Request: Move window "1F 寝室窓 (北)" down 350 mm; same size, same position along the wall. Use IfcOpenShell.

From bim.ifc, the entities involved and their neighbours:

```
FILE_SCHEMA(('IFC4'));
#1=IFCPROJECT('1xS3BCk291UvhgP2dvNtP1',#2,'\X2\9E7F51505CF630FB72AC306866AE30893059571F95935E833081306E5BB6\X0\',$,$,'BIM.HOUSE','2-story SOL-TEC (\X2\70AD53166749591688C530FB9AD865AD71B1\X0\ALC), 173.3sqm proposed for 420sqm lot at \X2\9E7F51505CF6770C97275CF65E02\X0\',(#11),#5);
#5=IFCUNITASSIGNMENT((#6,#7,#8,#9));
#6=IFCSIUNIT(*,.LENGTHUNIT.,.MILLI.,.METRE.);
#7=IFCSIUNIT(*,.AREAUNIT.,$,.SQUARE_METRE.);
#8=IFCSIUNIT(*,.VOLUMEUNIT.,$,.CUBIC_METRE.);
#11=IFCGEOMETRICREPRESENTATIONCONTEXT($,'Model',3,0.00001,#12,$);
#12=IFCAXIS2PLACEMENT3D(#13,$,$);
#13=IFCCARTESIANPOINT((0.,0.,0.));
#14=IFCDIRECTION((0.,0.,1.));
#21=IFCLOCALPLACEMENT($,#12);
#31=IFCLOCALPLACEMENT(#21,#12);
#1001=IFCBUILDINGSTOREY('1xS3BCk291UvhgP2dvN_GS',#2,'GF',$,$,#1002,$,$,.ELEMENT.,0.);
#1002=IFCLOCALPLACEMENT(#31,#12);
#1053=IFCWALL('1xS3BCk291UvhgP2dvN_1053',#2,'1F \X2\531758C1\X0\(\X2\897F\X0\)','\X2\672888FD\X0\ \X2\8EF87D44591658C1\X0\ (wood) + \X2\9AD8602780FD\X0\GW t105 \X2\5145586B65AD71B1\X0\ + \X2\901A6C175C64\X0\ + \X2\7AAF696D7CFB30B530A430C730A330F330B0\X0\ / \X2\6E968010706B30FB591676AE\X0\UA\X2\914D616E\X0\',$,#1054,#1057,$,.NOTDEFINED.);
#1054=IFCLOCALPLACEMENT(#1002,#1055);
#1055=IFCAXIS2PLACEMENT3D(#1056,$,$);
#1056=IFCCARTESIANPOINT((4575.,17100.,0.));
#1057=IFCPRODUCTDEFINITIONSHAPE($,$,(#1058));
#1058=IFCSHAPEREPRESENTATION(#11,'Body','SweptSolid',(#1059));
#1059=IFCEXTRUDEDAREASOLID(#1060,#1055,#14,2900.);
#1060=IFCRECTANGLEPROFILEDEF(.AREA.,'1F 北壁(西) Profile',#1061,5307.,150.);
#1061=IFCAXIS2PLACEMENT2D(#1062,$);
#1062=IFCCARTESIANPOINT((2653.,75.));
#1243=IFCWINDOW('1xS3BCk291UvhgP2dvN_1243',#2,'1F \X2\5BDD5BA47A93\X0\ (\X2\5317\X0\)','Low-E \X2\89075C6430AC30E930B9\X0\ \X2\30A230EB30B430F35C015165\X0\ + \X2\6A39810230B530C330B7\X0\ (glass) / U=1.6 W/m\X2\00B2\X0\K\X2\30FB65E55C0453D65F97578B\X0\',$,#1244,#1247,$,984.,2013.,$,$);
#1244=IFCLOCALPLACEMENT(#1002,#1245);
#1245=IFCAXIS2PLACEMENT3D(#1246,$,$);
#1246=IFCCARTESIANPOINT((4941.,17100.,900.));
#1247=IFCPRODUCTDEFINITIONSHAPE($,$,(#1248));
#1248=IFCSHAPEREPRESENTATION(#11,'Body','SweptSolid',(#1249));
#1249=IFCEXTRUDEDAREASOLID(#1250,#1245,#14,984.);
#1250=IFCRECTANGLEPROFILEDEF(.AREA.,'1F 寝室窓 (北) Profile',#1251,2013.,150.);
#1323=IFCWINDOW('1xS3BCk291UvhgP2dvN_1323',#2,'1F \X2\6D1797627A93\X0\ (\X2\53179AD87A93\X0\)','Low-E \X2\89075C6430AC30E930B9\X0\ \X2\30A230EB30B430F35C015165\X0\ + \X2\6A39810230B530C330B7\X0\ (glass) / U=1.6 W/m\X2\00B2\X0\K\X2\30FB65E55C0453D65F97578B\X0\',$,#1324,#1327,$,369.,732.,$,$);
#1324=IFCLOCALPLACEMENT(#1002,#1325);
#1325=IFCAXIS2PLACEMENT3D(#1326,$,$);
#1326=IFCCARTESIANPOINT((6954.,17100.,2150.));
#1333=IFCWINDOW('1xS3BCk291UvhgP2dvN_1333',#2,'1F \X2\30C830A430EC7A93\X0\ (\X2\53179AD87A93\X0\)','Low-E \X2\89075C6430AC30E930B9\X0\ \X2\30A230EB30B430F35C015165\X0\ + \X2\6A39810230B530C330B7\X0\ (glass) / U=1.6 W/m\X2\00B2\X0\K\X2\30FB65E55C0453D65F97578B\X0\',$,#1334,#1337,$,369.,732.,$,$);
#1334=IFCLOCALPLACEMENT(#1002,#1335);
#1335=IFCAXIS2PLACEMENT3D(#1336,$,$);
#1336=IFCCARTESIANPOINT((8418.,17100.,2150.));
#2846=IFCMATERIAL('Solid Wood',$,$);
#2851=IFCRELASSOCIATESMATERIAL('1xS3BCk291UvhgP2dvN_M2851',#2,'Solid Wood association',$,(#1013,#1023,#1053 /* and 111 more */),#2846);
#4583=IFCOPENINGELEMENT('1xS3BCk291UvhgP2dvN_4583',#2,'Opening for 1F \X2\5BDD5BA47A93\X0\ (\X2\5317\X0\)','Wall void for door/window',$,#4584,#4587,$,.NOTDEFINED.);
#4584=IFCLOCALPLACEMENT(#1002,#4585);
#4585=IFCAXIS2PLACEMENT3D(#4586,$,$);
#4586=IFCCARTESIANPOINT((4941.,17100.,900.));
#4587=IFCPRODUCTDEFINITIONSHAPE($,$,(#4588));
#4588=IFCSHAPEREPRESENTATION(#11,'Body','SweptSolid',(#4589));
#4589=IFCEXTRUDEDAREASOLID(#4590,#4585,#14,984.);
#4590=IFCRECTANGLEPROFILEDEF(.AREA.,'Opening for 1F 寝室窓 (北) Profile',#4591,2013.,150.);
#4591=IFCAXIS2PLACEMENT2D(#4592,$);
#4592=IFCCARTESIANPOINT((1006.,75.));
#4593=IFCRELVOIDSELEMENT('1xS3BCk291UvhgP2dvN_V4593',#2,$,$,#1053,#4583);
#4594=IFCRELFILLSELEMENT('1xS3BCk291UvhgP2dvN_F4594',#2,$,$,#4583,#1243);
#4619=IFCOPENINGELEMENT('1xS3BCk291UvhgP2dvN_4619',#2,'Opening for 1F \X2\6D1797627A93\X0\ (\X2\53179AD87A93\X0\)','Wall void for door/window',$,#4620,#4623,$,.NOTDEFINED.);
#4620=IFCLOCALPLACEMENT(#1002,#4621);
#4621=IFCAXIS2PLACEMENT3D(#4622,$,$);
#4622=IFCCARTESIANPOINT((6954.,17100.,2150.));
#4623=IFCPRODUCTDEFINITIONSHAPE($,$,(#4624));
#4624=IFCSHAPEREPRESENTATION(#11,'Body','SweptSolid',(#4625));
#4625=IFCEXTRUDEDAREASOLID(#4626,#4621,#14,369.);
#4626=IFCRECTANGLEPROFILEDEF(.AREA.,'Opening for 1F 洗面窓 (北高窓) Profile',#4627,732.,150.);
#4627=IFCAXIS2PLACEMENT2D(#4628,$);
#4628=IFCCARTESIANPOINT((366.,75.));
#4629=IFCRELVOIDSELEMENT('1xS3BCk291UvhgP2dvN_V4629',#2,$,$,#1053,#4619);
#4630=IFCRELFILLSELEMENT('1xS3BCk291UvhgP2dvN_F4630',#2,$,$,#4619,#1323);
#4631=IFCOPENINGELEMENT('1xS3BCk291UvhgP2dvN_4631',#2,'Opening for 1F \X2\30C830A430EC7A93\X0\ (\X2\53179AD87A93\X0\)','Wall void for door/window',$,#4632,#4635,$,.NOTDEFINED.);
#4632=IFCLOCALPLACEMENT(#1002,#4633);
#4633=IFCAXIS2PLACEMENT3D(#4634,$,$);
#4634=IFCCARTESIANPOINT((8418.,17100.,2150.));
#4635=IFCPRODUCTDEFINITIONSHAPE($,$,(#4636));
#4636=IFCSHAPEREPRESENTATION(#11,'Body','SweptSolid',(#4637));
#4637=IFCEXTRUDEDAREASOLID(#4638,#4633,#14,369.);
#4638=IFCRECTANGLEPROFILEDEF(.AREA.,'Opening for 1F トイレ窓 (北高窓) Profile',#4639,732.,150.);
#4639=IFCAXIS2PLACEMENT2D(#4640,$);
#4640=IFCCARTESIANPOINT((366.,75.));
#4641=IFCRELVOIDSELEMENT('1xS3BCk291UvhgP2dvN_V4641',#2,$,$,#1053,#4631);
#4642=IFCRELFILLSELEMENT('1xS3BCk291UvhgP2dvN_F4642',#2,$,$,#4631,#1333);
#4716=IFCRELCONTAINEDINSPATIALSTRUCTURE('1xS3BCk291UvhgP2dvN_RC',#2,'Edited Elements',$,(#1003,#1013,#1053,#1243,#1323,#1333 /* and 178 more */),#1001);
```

```python
import numpy as np
import ifcopenshell
import ifcopenshell.api.geometry
import ifcopenshell.util.placement
import ifcopenshell.util.unit

model = ifcopenshell.open("bim.ifc")
unit_scale = ifcopenshell.util.unit.calculate_unit_scale(model)

window = model.by_guid("1xS3BCk291UvhgP2dvN_1243")
opening = window.FillsVoids[0].RelatingOpeningElement
dz = -0.35 / unit_scale

shift = np.array([0.0, 0.0, dz])
# The window is not placed relative to its opening, so move both.
for product in (opening, window):
    matrix = ifcopenshell.util.placement.get_local_placement(product.ObjectPlacement)
    matrix[:3, 3] += shift
    ifcopenshell.api.geometry.edit_object_placement(model, product=product, matrix=matrix, is_si=False)

print(f"moved by {dz * unit_scale:+.3f} m")

model.write("bim_edited.ifc")
```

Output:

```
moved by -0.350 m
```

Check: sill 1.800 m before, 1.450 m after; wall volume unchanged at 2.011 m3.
